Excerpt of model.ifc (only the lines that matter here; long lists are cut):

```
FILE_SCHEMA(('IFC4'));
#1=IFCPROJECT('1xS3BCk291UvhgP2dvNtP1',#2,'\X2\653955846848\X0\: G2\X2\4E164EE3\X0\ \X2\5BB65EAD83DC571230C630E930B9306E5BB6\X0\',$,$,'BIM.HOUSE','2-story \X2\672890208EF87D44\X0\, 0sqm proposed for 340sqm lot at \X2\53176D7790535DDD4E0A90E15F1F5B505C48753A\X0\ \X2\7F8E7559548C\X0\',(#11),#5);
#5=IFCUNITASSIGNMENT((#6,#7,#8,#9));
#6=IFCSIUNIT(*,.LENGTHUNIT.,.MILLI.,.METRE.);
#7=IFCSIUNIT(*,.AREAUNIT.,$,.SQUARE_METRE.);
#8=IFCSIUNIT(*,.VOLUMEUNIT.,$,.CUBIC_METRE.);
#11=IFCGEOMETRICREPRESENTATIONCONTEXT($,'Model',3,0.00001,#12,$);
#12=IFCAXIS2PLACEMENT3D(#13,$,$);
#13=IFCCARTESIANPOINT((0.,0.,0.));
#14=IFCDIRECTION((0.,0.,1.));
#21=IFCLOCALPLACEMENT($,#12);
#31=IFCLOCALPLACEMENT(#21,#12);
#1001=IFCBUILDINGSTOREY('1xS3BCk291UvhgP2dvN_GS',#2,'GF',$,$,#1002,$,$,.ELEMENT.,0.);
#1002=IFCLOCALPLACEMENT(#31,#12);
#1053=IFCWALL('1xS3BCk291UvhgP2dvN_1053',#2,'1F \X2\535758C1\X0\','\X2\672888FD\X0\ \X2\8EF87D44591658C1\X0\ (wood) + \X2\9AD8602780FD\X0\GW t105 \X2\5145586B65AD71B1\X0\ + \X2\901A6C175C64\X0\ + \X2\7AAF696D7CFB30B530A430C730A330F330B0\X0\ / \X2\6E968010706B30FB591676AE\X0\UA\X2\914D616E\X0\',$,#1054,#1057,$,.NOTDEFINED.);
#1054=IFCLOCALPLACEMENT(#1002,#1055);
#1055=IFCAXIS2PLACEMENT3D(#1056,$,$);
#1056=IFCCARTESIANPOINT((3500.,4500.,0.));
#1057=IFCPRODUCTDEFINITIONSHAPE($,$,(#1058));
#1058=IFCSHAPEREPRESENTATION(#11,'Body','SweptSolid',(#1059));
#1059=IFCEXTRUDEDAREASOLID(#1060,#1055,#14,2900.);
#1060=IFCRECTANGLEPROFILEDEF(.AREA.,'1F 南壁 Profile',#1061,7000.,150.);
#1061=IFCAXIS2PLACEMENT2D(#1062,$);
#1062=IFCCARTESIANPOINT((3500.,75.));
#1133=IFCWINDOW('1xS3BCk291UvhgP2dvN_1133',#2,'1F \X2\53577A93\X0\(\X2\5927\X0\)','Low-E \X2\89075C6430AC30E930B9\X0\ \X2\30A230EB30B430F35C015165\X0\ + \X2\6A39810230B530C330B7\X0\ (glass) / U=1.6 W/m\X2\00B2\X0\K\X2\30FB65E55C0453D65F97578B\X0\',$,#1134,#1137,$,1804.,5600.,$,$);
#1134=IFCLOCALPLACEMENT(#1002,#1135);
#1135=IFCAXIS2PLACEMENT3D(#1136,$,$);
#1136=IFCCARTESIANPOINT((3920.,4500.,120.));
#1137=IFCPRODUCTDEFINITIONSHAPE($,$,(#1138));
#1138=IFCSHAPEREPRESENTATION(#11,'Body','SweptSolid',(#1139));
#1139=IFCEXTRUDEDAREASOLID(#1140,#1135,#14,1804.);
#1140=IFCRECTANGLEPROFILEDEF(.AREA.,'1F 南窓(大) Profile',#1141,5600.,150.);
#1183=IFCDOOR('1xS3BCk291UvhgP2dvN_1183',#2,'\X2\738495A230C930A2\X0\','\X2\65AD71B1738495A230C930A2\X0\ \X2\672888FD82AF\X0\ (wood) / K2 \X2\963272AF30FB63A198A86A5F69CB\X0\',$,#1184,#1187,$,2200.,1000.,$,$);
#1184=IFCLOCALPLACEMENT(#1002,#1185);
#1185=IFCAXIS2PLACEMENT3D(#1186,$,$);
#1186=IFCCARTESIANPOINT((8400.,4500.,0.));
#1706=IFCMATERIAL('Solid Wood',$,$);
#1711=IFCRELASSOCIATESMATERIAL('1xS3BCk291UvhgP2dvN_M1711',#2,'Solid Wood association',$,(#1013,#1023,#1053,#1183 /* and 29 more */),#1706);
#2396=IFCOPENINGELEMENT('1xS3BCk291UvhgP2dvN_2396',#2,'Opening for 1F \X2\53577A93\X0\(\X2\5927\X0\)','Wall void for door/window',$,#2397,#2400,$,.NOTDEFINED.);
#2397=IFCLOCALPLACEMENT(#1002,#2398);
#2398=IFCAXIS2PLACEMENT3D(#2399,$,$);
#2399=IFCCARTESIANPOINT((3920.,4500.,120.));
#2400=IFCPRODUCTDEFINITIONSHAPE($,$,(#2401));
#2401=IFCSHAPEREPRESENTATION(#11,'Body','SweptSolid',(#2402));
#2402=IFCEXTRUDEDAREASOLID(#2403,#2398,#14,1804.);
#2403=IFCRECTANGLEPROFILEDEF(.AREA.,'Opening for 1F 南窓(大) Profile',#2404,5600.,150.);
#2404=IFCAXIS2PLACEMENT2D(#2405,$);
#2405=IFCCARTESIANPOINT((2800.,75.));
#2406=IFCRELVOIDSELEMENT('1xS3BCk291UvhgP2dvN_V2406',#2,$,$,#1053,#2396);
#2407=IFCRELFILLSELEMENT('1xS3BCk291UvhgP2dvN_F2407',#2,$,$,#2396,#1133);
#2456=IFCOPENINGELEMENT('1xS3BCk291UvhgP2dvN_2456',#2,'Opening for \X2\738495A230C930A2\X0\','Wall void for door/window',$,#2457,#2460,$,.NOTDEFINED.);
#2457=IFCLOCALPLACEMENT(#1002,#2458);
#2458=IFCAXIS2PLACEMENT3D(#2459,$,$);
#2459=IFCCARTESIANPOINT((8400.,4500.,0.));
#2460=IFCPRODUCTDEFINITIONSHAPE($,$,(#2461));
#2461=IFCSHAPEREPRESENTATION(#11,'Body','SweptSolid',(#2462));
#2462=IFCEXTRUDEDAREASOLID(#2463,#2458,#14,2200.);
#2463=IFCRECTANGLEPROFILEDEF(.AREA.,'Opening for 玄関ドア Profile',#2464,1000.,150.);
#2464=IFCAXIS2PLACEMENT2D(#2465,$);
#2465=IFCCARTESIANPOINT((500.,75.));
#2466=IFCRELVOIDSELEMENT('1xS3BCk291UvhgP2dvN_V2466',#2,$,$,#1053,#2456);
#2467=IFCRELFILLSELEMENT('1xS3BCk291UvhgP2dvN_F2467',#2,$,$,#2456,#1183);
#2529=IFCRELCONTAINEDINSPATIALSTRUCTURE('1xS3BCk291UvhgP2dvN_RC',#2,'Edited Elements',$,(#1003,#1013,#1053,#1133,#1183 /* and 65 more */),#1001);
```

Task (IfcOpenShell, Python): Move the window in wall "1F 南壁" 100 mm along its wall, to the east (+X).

```python
import ifcopenshell
import ifcopenshell.api.geometry
import ifcopenshell.util.placement
import ifcopenshell.util.unit

model = ifcopenshell.open("model.ifc")
unit_scale = ifcopenshell.util.unit.calculate_unit_scale(model)

window = model.by_guid("1xS3BCk291UvhgP2dvN_1133")
opening = window.FillsVoids[0].RelatingOpeningElement
wall = opening.VoidsElements[0].RelatingBuildingElement

wall_matrix = ifcopenshell.util.placement.get_local_placement(wall.ObjectPlacement)
shift = wall_matrix[:3, 0] * 0.1 / unit_scale
before = ifcopenshell.util.placement.get_local_placement(window.ObjectPlacement)[:3, 3].copy()

# The window is not placed relative to its opening, so move both.
for product in (opening, window):
    matrix = ifcopenshell.util.placement.get_local_placement(product.ObjectPlacement)
    matrix[:3, 3] += shift
    ifcopenshell.api.geometry.edit_object_placement(model, product=product, matrix=matrix, is_si=False)

after = ifcopenshell.util.placement.get_local_placement(window.ObjectPlacement)[:3, 3]
print("window moved by", (after - before).round(3) + 0.0)

model.write("model_v2.ifc")
```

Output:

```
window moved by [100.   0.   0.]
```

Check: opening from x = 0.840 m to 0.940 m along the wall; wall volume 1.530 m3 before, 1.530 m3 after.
